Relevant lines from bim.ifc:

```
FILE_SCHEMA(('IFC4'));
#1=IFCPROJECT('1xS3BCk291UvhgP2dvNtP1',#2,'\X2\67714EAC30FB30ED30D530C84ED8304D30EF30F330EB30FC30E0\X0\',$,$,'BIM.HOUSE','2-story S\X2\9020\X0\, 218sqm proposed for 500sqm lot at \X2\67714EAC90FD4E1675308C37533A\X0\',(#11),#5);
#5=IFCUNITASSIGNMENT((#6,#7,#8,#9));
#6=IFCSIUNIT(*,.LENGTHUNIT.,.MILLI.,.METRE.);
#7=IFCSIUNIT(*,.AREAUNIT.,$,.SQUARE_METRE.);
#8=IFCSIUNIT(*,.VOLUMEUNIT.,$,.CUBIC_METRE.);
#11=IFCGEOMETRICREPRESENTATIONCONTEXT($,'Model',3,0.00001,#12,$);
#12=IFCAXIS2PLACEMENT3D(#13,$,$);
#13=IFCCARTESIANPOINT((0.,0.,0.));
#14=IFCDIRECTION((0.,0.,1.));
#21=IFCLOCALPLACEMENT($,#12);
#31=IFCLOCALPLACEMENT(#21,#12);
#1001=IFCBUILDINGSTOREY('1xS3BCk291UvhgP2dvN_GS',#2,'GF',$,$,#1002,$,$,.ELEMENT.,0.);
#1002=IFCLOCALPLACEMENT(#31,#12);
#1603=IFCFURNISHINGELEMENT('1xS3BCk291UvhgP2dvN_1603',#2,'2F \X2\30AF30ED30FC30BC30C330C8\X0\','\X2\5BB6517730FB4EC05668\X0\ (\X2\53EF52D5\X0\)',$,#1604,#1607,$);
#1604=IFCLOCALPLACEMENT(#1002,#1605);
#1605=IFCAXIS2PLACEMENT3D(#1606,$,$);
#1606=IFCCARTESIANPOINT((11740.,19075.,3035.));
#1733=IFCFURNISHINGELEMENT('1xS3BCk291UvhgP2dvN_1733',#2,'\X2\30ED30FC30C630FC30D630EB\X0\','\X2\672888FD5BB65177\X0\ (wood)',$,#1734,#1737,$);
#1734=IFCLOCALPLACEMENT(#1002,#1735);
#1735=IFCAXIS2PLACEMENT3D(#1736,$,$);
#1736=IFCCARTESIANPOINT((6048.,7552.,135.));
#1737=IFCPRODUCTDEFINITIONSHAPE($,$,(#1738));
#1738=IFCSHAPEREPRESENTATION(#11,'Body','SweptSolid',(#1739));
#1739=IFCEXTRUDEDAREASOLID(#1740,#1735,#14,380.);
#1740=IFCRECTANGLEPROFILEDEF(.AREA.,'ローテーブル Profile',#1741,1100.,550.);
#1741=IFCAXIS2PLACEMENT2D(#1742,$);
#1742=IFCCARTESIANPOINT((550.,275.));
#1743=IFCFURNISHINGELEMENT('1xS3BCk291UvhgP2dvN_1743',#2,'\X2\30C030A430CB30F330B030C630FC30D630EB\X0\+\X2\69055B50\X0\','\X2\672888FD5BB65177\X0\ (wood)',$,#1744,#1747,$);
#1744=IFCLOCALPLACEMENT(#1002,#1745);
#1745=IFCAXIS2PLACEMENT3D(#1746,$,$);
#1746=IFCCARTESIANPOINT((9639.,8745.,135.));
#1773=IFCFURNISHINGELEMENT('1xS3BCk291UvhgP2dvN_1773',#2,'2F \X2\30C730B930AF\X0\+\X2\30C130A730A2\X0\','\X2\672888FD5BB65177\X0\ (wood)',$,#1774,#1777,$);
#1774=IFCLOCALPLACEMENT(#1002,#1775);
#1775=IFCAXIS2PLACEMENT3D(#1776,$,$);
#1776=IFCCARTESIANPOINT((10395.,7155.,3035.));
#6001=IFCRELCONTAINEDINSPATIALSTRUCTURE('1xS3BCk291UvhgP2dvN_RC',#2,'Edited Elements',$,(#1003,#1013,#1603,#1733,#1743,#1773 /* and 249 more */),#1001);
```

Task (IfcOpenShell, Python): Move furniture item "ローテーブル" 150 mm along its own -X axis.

```python
import ifcopenshell
import ifcopenshell.api.geometry
import ifcopenshell.util.placement
import ifcopenshell.util.unit

model = ifcopenshell.open("bim.ifc")
unit_scale = ifcopenshell.util.unit.calculate_unit_scale(model)

item = model.by_guid("1xS3BCk291UvhgP2dvN_1733")
matrix = ifcopenshell.util.placement.get_local_placement(item.ObjectPlacement)
matrix[:3, 3] -= matrix[:3, 0] * 0.15 / unit_scale
ifcopenshell.api.geometry.edit_object_placement(model, product=item, matrix=matrix, is_si=False)

print(ifcopenshell.util.placement.get_local_placement(item.ObjectPlacement).round(3) + 0.0)

model.write("bim-out.ifc")
```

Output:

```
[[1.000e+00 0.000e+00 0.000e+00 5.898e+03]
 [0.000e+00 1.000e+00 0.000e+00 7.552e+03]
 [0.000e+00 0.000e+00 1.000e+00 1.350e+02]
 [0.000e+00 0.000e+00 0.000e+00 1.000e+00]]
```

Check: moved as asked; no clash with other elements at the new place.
